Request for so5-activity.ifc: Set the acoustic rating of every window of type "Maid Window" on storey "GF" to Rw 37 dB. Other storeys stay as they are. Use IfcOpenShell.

First a look at what the model holds.

```python
import ifcopenshell
import ifcopenshell.util.element

model = ifcopenshell.open("so5-activity.ifc")
print(model.schema)
storey = next(s for s in model.by_type("IfcBuildingStorey") if s.Name == "GF")
windows = [e for e in ifcopenshell.util.element.get_decomposition(storey) if e.is_a("IfcWindow")]
seen = {}
for e in windows:
    element_type = ifcopenshell.util.element.get_type(e)
    key = (element_type.Name if element_type != e and element_type else None, ifcopenshell.util.element.get_pset(e, "Pset_WindowCommon", "AcousticRating"))
    seen[key] = seen.get(key, 0) + 1
for (name, value), count in sorted(seen.items(), key=str):
    print(count, "x", name, "|", value)
```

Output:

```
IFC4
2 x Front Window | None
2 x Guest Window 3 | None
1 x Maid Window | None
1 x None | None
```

```python
import ifcopenshell
import ifcopenshell.api.pset
import ifcopenshell.util.element

model = ifcopenshell.open("so5-activity.ifc")

storey = next(s for s in model.by_type("IfcBuildingStorey") if s.Name == "GF")
windows = [e for e in ifcopenshell.util.element.get_decomposition(storey) if e.is_a("IfcWindow")]

count = 0
for e in windows:
    element_type = ifcopenshell.util.element.get_type(e)
    if element_type in (None, e) or element_type.Name != "Maid Window":
        continue
    # add_pset returns the element's existing set when there is one.
    pset = ifcopenshell.api.pset.add_pset(model, product=e, name="Pset_WindowCommon")
    ifcopenshell.api.pset.edit_pset(model, pset=pset, properties={"AcousticRating": "Rw 37 dB"})
    count += 1

print(count, "windows updated")

model.write("so5-activity-out.ifc")
```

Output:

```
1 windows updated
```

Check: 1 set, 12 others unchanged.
